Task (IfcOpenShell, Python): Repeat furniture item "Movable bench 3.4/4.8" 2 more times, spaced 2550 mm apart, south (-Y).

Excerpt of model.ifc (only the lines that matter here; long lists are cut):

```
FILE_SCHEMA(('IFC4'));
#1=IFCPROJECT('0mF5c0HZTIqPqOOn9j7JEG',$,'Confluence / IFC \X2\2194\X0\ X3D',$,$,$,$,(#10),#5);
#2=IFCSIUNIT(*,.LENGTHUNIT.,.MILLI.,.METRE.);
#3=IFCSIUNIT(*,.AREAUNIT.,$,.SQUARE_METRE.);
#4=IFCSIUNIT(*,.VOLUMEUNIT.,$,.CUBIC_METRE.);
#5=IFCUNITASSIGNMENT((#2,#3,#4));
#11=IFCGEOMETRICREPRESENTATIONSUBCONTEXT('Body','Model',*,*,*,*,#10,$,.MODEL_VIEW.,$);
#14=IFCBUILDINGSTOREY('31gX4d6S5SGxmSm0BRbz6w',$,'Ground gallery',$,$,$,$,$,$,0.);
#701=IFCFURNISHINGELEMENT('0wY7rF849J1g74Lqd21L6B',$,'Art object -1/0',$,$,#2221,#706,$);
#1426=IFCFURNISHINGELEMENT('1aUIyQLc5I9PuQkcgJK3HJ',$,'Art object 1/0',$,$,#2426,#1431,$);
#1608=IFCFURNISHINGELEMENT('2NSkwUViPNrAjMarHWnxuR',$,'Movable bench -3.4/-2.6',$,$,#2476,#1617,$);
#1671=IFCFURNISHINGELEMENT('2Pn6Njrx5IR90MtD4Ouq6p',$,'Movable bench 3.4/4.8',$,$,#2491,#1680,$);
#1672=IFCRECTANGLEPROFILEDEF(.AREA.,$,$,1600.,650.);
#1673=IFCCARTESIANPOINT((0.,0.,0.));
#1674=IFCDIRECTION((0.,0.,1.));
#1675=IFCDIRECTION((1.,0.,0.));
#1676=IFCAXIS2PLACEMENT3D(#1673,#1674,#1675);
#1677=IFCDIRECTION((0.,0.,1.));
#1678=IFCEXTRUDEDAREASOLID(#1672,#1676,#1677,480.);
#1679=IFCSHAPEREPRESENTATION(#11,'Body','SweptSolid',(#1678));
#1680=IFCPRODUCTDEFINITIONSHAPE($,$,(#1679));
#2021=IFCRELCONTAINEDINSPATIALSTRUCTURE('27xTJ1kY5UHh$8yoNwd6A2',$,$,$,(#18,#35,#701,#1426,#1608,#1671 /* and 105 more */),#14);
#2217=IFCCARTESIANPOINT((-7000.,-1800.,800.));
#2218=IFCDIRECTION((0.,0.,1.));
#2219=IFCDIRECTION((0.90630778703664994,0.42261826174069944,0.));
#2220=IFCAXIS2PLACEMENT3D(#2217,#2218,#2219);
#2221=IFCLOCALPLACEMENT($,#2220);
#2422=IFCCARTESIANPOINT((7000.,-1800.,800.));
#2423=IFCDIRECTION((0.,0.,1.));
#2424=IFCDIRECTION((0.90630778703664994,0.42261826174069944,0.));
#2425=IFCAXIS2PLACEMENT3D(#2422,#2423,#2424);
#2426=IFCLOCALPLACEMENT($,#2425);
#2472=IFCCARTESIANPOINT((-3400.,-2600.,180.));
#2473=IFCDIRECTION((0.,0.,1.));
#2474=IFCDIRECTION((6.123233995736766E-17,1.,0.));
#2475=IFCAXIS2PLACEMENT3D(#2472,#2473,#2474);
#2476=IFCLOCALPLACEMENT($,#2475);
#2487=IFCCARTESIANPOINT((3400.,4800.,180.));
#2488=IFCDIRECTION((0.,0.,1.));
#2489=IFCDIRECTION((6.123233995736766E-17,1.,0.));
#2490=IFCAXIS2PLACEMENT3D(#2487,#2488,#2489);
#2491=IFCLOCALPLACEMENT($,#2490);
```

```python
import numpy as np
import ifcopenshell
import ifcopenshell.api.geometry
import ifcopenshell.api.root
import ifcopenshell.util.element
import ifcopenshell.util.placement
import ifcopenshell.util.unit

model = ifcopenshell.open("model.ifc")
unit_scale = ifcopenshell.util.unit.calculate_unit_scale(model)

source = model.by_id(1671)
base = ifcopenshell.util.placement.get_local_placement(source.ObjectPlacement)
step = np.array([0.0, -1.0, 0.0]) * 2.55 / unit_scale

for i in range(1, 3):
    copy = ifcopenshell.api.root.copy_class(model, product=source)
    copy.Representation = ifcopenshell.util.element.copy_deep(
        model, source.Representation, exclude=["IfcGeometricRepresentationContext", "IfcRepresentationMap"]
    )
    matrix = base.copy()
    matrix[:3, 3] += i * step
    print("added at", matrix[:3, 3].round(3) + 0.0)
    ifcopenshell.api.geometry.edit_object_placement(model, product=copy, matrix=matrix, is_si=False)

model.write("model_edited.ifc")
```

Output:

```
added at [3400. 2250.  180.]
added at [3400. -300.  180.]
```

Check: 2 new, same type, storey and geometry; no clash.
